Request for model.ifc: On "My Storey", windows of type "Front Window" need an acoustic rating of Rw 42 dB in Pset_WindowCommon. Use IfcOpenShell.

First a look at what the model holds.

```python
import ifcopenshell
import ifcopenshell.util.element

model = ifcopenshell.open("model.ifc")
print(model.schema)
storey = next(s for s in model.by_type("IfcBuildingStorey") if s.Name == "My Storey")
windows = [e for e in ifcopenshell.util.element.get_decomposition(storey) if e.is_a("IfcWindow")]
seen = {}
for e in windows:
    element_type = ifcopenshell.util.element.get_type(e)
    key = (element_type.Name if element_type != e and element_type else None, ifcopenshell.util.element.get_pset(e, "Pset_WindowCommon", "AcousticRating"))
    seen[key] = seen.get(key, 0) + 1
for (name, value), count in sorted(seen.items(), key=str):
    print(count, "x", name, "|", value)
```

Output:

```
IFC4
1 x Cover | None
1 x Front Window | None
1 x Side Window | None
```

```python
import ifcopenshell
import ifcopenshell.api.pset
import ifcopenshell.util.element

model = ifcopenshell.open("model.ifc")

storey = next(s for s in model.by_type("IfcBuildingStorey") if s.Name == "My Storey")
windows = [e for e in ifcopenshell.util.element.get_decomposition(storey) if e.is_a("IfcWindow")]

count = 0
for e in windows:
    element_type = ifcopenshell.util.element.get_type(e)
    if element_type in (None, e) or element_type.Name != "Front Window":
        continue
    # add_pset returns the element's existing set when there is one.
    pset = ifcopenshell.api.pset.add_pset(model, product=e, name="Pset_WindowCommon")
    ifcopenshell.api.pset.edit_pset(model, pset=pset, properties={"AcousticRating": "Rw 42 dB"})
    count += 1

print(count, "windows updated")

model.write("model_updated.ifc")
```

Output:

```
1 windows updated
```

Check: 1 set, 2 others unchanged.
